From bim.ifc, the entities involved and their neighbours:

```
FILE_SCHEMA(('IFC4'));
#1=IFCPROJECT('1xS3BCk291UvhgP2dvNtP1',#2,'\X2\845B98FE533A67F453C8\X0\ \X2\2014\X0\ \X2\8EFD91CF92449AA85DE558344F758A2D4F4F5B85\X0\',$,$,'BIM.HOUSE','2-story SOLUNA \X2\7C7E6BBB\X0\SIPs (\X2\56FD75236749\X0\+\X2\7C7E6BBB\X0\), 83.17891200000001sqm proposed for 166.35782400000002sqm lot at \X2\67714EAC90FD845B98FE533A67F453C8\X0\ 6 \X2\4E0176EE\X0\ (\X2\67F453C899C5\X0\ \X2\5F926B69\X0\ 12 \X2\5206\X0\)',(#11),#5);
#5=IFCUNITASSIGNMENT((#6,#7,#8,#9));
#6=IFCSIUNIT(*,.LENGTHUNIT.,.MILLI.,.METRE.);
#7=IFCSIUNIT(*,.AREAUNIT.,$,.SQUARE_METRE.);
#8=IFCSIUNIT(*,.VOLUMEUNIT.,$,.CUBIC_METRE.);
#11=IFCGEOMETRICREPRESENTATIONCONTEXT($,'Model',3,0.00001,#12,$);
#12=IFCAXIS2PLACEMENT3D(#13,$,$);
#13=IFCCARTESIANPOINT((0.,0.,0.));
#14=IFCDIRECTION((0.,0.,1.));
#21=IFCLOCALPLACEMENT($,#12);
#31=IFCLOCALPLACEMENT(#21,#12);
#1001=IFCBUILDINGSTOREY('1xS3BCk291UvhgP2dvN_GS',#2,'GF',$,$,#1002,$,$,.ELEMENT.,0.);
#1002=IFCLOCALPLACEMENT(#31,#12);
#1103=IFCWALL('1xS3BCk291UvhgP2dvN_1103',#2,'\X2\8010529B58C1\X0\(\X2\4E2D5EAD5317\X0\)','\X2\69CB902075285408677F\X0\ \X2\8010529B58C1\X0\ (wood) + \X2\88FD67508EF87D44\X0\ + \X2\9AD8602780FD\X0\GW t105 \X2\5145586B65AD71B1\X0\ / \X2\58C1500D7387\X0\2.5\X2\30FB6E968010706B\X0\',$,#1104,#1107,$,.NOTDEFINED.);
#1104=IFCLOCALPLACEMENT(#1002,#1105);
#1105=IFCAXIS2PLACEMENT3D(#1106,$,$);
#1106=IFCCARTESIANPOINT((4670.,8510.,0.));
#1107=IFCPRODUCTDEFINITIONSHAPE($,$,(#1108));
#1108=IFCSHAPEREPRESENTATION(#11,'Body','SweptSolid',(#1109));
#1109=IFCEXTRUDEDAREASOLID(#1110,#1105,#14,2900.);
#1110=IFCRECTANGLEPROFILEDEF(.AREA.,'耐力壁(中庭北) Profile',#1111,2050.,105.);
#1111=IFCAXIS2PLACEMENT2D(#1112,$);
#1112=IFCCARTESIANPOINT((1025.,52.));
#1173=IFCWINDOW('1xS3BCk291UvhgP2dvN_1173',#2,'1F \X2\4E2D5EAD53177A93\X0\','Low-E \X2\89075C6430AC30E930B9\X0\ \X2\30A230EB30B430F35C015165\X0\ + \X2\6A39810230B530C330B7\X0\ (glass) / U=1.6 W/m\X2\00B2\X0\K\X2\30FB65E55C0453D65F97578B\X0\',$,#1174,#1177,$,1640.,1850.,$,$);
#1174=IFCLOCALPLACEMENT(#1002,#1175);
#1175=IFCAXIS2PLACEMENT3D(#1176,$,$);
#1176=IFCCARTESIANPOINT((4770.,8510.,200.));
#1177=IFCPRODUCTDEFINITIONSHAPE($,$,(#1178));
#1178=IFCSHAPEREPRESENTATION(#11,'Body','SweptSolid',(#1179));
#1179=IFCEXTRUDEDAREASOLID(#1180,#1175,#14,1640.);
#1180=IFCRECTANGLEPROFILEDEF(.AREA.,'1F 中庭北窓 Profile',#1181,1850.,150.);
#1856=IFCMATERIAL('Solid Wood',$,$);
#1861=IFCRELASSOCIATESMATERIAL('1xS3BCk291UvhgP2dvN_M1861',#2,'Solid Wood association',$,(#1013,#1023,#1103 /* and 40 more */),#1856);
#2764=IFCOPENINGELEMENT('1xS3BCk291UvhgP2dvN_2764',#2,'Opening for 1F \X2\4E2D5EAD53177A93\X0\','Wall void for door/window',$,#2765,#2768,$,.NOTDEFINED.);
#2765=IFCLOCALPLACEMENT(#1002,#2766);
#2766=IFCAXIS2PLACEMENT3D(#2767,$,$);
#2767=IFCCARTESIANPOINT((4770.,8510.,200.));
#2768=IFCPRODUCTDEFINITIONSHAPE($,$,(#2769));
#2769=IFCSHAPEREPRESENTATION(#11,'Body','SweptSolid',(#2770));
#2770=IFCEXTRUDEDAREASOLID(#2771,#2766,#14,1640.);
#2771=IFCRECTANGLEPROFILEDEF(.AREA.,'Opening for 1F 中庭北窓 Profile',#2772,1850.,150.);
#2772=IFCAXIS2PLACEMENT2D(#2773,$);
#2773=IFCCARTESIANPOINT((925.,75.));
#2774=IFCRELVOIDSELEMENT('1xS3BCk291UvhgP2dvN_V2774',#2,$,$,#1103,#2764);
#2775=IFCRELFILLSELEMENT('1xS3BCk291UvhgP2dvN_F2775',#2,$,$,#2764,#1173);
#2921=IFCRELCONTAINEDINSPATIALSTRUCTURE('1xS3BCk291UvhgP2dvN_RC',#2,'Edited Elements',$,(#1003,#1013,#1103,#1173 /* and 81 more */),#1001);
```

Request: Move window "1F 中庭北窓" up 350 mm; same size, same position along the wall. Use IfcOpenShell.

```python
import numpy as np
import ifcopenshell
import ifcopenshell.api.geometry
import ifcopenshell.util.placement
import ifcopenshell.util.unit

model = ifcopenshell.open("bim.ifc")
unit_scale = ifcopenshell.util.unit.calculate_unit_scale(model)

window = model.by_id(1173)
opening = window.FillsVoids[0].RelatingOpeningElement
dz = 350.0

shift = np.array([0.0, 0.0, dz])
# The window is not placed relative to its opening, so move both.
for product in (opening, window):
    matrix = ifcopenshell.util.placement.get_local_placement(product.ObjectPlacement)
    matrix[:3, 3] += shift
    ifcopenshell.api.geometry.edit_object_placement(model, product=product, matrix=matrix, is_si=False)

print(f"moved by {dz * unit_scale:+.3f} m")

model.write("bim-out.ifc")
```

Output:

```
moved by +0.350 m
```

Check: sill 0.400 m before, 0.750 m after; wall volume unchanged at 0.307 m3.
